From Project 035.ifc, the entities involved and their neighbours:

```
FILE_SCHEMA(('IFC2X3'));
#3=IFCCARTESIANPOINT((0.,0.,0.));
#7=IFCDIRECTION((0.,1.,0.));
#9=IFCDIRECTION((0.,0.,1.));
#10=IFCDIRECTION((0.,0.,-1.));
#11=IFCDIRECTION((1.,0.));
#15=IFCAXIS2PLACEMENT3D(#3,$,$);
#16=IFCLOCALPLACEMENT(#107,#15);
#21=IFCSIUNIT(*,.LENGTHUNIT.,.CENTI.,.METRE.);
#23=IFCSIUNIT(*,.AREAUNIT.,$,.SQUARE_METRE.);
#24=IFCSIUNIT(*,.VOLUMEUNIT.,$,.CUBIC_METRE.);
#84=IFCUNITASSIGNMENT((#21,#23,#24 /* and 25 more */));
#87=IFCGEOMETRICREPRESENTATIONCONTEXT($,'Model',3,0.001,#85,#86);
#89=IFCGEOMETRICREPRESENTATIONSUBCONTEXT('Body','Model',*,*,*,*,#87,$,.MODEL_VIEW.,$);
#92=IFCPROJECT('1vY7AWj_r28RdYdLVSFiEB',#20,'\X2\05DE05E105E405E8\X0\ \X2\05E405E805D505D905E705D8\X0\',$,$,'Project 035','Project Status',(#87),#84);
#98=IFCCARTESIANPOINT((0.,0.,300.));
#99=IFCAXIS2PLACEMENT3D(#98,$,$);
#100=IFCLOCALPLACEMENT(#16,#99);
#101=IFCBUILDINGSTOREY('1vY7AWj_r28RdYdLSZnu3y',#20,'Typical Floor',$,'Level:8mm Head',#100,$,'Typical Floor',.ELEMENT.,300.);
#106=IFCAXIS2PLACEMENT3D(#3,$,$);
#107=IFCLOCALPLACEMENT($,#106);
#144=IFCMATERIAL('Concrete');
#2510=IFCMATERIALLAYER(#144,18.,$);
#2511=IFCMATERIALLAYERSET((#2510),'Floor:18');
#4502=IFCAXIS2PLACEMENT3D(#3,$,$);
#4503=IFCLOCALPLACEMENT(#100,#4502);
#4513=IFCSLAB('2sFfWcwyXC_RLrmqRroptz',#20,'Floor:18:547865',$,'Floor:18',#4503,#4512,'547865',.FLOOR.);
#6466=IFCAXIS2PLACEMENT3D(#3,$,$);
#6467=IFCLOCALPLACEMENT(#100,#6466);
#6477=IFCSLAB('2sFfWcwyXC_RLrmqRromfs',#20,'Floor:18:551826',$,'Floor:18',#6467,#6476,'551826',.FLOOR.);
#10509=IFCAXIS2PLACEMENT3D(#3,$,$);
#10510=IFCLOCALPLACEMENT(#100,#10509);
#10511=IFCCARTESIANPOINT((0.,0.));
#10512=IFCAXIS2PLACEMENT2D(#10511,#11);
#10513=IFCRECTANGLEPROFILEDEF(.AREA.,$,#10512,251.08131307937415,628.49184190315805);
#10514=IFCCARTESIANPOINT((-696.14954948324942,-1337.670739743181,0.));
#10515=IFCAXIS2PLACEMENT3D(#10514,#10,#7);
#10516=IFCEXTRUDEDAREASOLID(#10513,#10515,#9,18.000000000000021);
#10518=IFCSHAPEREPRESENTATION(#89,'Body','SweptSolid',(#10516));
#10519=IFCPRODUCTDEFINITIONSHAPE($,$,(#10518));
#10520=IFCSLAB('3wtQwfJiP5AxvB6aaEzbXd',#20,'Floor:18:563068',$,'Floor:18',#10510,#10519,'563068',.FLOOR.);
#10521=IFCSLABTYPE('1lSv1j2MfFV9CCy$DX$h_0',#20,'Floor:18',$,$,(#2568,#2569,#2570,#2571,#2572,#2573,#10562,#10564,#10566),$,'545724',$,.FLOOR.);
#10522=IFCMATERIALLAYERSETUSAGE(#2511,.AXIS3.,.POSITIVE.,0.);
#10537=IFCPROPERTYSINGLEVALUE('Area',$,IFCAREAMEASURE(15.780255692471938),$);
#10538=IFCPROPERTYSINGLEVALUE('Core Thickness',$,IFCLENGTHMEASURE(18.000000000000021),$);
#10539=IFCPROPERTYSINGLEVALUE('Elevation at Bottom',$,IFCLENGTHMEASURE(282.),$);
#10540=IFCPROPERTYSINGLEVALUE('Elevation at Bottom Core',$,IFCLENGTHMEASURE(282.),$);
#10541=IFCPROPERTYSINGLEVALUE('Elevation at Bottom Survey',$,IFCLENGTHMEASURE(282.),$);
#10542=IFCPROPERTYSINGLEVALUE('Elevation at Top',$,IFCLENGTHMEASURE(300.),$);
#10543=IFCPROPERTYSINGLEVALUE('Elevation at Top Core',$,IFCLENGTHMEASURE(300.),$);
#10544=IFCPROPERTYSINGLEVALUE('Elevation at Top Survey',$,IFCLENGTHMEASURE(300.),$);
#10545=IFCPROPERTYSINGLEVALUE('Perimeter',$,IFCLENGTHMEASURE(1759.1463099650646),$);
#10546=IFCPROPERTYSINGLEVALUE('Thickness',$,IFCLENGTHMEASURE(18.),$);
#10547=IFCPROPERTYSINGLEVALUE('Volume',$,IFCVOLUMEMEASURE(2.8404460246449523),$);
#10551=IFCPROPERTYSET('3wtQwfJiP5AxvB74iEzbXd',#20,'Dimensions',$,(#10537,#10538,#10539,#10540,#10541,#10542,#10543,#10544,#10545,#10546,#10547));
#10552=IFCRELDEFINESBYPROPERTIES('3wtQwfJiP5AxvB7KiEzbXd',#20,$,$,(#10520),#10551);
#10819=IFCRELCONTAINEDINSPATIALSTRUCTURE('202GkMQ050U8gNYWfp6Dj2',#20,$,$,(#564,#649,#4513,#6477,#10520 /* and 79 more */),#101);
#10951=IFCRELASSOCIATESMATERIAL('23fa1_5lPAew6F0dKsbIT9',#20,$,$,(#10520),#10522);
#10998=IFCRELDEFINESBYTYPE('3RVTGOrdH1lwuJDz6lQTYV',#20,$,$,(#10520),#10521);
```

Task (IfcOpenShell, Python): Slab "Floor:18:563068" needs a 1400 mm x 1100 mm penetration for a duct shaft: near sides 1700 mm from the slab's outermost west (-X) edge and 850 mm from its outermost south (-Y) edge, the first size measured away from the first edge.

```python
import numpy as np
import ifcopenshell
import ifcopenshell.api.feature
import ifcopenshell.api.geometry
import ifcopenshell.api.pset
import ifcopenshell.api.root
import ifcopenshell.geom
import ifcopenshell.util.element
import ifcopenshell.util.placement
import ifcopenshell.util.representation
import ifcopenshell.util.shape
import ifcopenshell.util.unit

model = ifcopenshell.open("Project 035.ifc")
unit_scale = ifcopenshell.util.unit.calculate_unit_scale(model)
area_scale = ifcopenshell.util.unit.calculate_unit_scale(model, "AREAUNIT")
volume_scale = ifcopenshell.util.unit.calculate_unit_scale(model, "VOLUMEUNIT")
settings = ifcopenshell.geom.settings()


def volume(element):
    """Net volume in cubic metres, openings subtracted."""
    shape = ifcopenshell.geom.create_shape(settings, element)
    return ifcopenshell.util.shape.get_volume(shape.geometry)


slab = model.by_guid("3wtQwfJiP5AxvB6aaEzbXd")
before = volume(slab)

# Extent in the slab's own axes, in metres. The edges named are its -X and -Y sides.
slab_shape = ifcopenshell.geom.create_shape(settings, slab)
vertices = ifcopenshell.util.shape.get_vertices(slab_shape.geometry)
x_min, y_min, bottom = vertices.min(axis=0)
top = vertices[:, 2].max()

opening = ifcopenshell.api.root.create_entity(model, ifc_class="IfcOpeningElement", name="Duct shaft opening")
context = ifcopenshell.util.representation.get_context(model, "Model", "Body", "MODEL_VIEW")
width, depth = 1.4, 1.1
outline = [(0.0, 0.0), (width, 0.0), (width, depth), (0.0, depth), (0.0, 0.0)]
# Overshoot both faces by 50 mm so the cut is clean.
shape = ifcopenshell.api.geometry.add_slab_representation(
    model, context=context, depth=top - bottom + 0.1, polyline=outline
)
ifcopenshell.api.geometry.assign_representation(model, product=opening, representation=shape)

matrix = ifcopenshell.util.placement.get_local_placement(slab.ObjectPlacement)
matrix[:, 3] = matrix @ np.append(np.array([x_min + 1.7, y_min + 0.85, bottom - 0.05]) / unit_scale, 1.0)
ifcopenshell.api.geometry.edit_object_placement(model, product=opening, matrix=matrix, is_si=False)
ifcopenshell.api.feature.add_feature(model, feature=opening, element=slab)

after = volume(slab)

# Update the slab's stored quantities.
pset = model.by_id(ifcopenshell.util.element.get_pset(slab, "Dimensions", should_inherit=False)["id"])
ifcopenshell.api.pset.edit_pset(model, pset=pset, properties={
    "Area": model.create_entity("IfcAreaMeasure", after / (top - bottom) / area_scale),
    "Volume": model.create_entity("IfcVolumeMeasure", after / volume_scale),
})

print(f"slab volume {before:.3f} -> {after:.3f} m3")

model.write("Project 035_edited.ifc")
```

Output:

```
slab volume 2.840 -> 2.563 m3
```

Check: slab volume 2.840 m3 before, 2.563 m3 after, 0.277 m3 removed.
